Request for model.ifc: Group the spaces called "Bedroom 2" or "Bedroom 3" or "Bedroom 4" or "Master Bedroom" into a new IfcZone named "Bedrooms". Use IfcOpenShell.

First a look at what the model holds.

```python
import ifcopenshell

model = ifcopenshell.open("model.ifc")
print(model.schema)
seen = {}
for space in model.by_type("IfcSpace"):
    seen[space.LongName] = seen.get(space.LongName, 0) + 1
for name, count in sorted(seen.items(), key=str):
    print(count, "x", name)
print("zones:", [z.Name for z in model.by_type("IfcZone")][:20])
```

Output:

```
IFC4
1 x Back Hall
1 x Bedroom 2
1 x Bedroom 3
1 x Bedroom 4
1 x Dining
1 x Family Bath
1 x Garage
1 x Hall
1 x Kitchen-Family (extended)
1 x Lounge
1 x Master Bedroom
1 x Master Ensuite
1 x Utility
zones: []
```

```python
import ifcopenshell
import ifcopenshell.api.group
import ifcopenshell.api.root

model = ifcopenshell.open("model.ifc")

names = {"Bedroom 2", "Bedroom 3", "Bedroom 4", "Master Bedroom"}
spaces = [s for s in model.by_type("IfcSpace") if s.LongName in names]

zone = ifcopenshell.api.root.create_entity(model, ifc_class="IfcZone", name="Bedrooms")
ifcopenshell.api.group.assign_group(model, products=spaces, group=zone)
print(len(spaces), "spaces in", zone.Name)

model.write("model_updated.ifc")
```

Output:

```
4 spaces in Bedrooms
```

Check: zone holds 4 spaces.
